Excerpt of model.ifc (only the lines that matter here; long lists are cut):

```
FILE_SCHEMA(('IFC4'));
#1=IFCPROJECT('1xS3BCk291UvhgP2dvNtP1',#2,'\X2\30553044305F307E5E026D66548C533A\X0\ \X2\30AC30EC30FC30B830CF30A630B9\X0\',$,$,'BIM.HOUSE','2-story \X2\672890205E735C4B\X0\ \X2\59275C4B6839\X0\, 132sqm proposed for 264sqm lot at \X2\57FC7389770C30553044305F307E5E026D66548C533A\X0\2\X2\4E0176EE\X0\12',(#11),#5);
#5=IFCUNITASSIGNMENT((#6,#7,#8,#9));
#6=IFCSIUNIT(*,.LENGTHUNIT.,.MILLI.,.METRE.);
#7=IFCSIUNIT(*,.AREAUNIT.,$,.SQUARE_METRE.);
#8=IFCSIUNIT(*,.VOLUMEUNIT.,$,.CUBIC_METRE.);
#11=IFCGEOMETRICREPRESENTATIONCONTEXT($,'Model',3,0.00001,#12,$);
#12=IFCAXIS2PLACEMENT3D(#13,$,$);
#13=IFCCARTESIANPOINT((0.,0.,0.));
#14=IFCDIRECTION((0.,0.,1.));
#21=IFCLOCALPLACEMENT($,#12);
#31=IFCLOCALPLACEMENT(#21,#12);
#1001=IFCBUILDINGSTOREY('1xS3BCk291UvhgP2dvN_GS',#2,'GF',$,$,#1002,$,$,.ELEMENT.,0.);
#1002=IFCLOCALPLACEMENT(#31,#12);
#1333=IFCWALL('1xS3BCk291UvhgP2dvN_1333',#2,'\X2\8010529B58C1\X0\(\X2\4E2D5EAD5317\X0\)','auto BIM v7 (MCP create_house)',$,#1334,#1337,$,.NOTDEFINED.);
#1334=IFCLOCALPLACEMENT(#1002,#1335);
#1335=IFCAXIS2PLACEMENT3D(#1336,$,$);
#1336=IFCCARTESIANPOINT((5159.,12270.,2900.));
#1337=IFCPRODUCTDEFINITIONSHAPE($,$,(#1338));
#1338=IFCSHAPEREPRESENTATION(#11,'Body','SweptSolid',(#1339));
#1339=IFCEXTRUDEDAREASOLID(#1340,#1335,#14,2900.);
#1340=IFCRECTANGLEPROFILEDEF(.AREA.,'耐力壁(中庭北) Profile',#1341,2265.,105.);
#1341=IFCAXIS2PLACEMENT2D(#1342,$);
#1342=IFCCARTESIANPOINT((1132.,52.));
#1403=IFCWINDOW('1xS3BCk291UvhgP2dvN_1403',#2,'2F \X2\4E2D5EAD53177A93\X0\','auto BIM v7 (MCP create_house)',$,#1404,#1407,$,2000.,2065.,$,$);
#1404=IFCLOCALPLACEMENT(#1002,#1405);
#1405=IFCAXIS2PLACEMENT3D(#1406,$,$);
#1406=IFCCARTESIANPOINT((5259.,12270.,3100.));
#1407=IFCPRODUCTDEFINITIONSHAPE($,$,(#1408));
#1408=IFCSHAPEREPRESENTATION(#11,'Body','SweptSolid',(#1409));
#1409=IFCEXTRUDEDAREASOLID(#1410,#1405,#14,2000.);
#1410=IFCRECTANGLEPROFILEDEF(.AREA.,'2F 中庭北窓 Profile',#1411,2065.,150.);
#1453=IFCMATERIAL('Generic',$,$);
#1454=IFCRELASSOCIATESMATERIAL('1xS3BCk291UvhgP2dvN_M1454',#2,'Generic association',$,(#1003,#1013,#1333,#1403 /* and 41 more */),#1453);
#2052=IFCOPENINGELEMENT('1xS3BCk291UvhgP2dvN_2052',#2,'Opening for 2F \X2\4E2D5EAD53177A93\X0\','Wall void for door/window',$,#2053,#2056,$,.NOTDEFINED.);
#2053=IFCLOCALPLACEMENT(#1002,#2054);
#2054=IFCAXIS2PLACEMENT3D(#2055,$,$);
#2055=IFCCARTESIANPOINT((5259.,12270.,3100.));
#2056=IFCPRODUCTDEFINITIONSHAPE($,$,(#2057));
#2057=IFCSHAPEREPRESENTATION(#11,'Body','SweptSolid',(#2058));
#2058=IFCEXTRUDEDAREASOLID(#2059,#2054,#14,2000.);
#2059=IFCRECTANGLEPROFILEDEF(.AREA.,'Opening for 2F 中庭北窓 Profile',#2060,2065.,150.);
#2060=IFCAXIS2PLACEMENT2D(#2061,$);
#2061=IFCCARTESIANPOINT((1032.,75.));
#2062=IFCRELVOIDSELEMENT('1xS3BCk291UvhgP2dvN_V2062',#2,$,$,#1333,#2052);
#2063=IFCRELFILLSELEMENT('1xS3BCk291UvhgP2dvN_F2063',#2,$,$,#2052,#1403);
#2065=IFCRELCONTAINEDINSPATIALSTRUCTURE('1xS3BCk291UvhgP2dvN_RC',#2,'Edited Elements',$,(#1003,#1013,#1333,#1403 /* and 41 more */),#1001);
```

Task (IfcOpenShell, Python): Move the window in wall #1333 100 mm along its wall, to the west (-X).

```python
import ifcopenshell
import ifcopenshell.api.geometry
import ifcopenshell.util.placement

model = ifcopenshell.open("model.ifc")

window = model.by_guid("1xS3BCk291UvhgP2dvN_1403")
opening = window.FillsVoids[0].RelatingOpeningElement
wall = opening.VoidsElements[0].RelatingBuildingElement

wall_matrix = ifcopenshell.util.placement.get_local_placement(wall.ObjectPlacement)
shift = wall_matrix[:3, 0] * -100.0
before = ifcopenshell.util.placement.get_local_placement(window.ObjectPlacement)[:3, 3].copy()

# The window is not placed relative to its opening, so move both.
for product in (opening, window):
    matrix = ifcopenshell.util.placement.get_local_placement(product.ObjectPlacement)
    matrix[:3, 3] += shift
    ifcopenshell.api.geometry.edit_object_placement(model, product=product, matrix=matrix, is_si=False)

after = ifcopenshell.util.placement.get_local_placement(window.ObjectPlacement)[:3, 3]
print("window moved by", (after - before).round(3) + 0.0)

model.write("model_updated.ifc")
```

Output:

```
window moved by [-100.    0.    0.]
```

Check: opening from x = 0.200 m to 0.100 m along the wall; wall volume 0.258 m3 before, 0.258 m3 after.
